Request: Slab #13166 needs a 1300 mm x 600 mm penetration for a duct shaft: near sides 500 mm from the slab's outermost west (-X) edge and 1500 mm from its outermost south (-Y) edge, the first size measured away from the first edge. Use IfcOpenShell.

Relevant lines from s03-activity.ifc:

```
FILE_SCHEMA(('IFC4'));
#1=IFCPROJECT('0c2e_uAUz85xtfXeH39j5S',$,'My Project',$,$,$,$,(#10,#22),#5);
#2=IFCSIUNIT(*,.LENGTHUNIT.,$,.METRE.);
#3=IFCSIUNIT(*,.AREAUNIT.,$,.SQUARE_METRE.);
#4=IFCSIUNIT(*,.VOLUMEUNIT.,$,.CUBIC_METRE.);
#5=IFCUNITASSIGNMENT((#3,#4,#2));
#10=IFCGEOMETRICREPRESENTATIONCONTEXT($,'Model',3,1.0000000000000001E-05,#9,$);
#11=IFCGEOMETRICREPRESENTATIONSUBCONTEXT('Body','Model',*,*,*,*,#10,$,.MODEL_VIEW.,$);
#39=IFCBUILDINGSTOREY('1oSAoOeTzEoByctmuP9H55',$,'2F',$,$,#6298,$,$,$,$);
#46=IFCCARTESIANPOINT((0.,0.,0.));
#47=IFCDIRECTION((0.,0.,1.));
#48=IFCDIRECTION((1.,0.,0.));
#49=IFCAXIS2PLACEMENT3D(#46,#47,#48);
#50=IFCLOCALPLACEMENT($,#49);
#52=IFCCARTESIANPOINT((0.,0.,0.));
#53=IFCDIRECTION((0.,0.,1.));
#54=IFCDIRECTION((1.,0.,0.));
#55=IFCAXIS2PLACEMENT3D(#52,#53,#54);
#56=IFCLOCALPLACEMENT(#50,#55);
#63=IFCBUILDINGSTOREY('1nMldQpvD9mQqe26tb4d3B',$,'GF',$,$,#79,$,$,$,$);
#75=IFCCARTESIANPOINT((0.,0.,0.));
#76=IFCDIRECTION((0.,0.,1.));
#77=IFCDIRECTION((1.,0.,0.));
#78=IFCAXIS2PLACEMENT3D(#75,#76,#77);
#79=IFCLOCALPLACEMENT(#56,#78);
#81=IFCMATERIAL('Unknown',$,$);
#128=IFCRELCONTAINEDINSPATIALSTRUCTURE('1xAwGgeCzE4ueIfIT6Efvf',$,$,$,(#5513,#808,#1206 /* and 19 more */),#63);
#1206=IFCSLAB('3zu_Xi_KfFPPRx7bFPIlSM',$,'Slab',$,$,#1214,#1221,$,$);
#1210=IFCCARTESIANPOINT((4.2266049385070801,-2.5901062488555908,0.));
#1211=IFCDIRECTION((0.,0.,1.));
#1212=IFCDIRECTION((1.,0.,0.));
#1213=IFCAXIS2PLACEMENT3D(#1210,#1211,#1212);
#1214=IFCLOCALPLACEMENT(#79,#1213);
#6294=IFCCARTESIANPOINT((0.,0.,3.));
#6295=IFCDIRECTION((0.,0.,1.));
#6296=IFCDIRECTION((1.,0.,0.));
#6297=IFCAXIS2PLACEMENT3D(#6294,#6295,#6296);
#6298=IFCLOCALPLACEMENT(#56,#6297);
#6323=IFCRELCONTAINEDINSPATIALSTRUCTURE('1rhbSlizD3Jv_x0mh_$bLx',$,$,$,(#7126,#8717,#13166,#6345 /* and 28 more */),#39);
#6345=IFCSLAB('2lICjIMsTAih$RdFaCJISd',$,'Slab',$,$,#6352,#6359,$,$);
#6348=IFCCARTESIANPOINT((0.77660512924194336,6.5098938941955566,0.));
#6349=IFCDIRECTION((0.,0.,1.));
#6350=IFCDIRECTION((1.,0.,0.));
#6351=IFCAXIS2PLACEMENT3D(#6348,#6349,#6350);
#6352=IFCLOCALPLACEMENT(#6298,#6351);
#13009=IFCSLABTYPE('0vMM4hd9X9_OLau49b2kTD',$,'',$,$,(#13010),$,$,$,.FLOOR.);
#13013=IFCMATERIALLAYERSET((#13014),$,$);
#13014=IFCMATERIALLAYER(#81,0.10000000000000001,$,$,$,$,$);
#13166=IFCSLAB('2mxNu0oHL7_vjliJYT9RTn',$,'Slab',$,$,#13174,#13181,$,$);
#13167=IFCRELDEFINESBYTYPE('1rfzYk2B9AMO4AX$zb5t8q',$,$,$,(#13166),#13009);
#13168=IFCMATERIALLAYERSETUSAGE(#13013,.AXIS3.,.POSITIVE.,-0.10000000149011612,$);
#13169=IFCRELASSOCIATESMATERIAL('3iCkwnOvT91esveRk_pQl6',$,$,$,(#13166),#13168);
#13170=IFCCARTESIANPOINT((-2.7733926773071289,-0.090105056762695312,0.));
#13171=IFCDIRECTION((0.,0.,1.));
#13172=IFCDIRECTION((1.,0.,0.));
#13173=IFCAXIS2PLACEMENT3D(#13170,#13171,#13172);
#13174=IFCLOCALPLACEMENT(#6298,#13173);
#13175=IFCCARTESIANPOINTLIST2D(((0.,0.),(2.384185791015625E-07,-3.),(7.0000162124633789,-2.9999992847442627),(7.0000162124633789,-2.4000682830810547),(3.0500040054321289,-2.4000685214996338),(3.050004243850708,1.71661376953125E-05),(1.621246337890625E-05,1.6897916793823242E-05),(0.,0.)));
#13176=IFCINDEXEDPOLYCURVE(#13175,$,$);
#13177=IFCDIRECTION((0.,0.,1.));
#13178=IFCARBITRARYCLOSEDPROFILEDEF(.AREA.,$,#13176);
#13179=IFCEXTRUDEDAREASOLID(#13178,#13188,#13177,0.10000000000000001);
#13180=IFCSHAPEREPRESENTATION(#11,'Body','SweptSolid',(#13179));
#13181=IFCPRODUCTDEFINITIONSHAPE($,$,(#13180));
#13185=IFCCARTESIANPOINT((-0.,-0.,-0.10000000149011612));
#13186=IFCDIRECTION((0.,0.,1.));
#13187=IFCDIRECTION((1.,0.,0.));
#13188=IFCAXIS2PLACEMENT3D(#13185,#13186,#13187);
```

```python
import numpy as np
import ifcopenshell
import ifcopenshell.api.feature
import ifcopenshell.api.geometry
import ifcopenshell.api.root
import ifcopenshell.geom
import ifcopenshell.util.placement
import ifcopenshell.util.representation
import ifcopenshell.util.shape
import ifcopenshell.util.unit

model = ifcopenshell.open("s03-activity.ifc")
unit_scale = ifcopenshell.util.unit.calculate_unit_scale(model)
settings = ifcopenshell.geom.settings()


def volume(element):
    """Net volume in cubic metres, openings subtracted."""
    shape = ifcopenshell.geom.create_shape(settings, element)
    return ifcopenshell.util.shape.get_volume(shape.geometry)


slab = model.by_id(13166)
before = volume(slab)

# Extent in the slab's own axes, in metres. The edges named are its -X and -Y sides.
slab_shape = ifcopenshell.geom.create_shape(settings, slab)
vertices = ifcopenshell.util.shape.get_vertices(slab_shape.geometry)
x_min, y_min, bottom = vertices.min(axis=0)
top = vertices[:, 2].max()

opening = ifcopenshell.api.root.create_entity(model, ifc_class="IfcOpeningElement", name="Duct shaft opening", predefined_type="OPENING")
context = ifcopenshell.util.representation.get_context(model, "Model", "Body", "MODEL_VIEW")
width, depth = 1.3, 0.6
outline = [(0.0, 0.0), (width, 0.0), (width, depth), (0.0, depth), (0.0, 0.0)]
# Overshoot both faces by 50 mm so the cut is clean.
shape = ifcopenshell.api.geometry.add_slab_representation(
    model, context=context, depth=top - bottom + 0.1, polyline=outline
)
ifcopenshell.api.geometry.assign_representation(model, product=opening, representation=shape)

matrix = ifcopenshell.util.placement.get_local_placement(slab.ObjectPlacement)
matrix[:, 3] = matrix @ np.append(np.array([x_min + 0.5, y_min + 1.5, bottom - 0.05]) / unit_scale, 1.0)
ifcopenshell.api.geometry.edit_object_placement(model, product=opening, matrix=matrix, is_si=False)
ifcopenshell.api.feature.add_feature(model, feature=opening, element=slab)

after = volume(slab)

print(f"slab volume {before:.3f} -> {after:.3f} m3")

model.write("s03-activity-out.ifc")
```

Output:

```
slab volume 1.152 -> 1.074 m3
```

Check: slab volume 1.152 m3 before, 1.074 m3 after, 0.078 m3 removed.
